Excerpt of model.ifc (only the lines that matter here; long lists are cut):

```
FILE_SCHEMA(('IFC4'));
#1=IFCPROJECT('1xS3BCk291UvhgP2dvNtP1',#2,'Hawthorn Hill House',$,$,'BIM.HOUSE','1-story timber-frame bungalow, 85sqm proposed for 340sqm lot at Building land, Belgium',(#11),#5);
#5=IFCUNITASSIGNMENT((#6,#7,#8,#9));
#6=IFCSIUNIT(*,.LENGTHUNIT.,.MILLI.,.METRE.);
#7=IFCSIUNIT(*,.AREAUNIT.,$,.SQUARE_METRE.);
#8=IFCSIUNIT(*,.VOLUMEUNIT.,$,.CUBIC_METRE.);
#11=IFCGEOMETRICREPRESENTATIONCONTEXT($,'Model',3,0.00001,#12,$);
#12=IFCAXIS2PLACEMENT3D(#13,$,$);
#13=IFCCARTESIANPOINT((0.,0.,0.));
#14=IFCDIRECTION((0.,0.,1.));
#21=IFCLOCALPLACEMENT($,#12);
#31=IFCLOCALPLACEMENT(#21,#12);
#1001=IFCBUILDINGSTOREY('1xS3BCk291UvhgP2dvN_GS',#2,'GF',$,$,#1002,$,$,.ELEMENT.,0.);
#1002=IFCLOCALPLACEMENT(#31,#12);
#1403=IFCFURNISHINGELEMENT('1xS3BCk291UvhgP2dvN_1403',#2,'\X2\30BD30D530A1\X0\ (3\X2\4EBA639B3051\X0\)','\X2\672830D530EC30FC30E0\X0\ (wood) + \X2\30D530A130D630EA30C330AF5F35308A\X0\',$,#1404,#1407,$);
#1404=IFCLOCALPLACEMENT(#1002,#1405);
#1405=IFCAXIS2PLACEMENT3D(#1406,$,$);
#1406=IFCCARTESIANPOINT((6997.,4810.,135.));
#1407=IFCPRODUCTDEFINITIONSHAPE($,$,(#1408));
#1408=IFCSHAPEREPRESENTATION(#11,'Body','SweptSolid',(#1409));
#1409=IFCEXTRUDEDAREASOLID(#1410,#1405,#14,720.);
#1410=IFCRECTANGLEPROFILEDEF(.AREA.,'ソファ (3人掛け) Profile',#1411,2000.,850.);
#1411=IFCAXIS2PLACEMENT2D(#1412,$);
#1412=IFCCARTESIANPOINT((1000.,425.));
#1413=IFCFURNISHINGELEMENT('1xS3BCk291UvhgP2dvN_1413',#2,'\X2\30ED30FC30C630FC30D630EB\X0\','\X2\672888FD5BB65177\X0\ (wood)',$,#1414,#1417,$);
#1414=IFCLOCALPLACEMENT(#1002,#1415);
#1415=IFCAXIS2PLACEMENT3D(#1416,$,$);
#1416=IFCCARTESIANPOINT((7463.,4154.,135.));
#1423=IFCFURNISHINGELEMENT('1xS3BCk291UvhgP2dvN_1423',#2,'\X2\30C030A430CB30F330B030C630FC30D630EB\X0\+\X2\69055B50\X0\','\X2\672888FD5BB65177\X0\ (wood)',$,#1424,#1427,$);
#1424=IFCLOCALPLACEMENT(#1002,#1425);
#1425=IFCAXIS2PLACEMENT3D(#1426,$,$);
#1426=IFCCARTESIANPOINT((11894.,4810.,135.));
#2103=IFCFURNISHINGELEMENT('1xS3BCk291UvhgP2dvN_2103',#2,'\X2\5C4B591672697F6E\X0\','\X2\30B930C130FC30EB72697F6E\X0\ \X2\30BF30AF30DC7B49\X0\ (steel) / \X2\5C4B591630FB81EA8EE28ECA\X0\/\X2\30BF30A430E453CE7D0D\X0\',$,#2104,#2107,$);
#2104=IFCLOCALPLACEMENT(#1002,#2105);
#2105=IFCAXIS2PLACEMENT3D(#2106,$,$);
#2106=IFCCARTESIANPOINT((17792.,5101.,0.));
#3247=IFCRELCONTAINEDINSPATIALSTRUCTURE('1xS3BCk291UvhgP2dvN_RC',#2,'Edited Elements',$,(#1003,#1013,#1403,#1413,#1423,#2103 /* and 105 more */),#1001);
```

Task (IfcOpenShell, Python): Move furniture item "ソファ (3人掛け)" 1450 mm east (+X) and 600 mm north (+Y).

```python
import ifcopenshell
import ifcopenshell.api.geometry
import ifcopenshell.util.placement
import ifcopenshell.util.unit

model = ifcopenshell.open("model.ifc")
unit_scale = ifcopenshell.util.unit.calculate_unit_scale(model)

item = model.by_id(1403)
matrix = ifcopenshell.util.placement.get_local_placement(item.ObjectPlacement)
matrix[0, 3] += 1.45 / unit_scale
matrix[1, 3] += 0.6 / unit_scale
ifcopenshell.api.geometry.edit_object_placement(model, product=item, matrix=matrix, is_si=False)

print(ifcopenshell.util.placement.get_local_placement(item.ObjectPlacement).round(3) + 0.0)

model.write("model-out.ifc")
```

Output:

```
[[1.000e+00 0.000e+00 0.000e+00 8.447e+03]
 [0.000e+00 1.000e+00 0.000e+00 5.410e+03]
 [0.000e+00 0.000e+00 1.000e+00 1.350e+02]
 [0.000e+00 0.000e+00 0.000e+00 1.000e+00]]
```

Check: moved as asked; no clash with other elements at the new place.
